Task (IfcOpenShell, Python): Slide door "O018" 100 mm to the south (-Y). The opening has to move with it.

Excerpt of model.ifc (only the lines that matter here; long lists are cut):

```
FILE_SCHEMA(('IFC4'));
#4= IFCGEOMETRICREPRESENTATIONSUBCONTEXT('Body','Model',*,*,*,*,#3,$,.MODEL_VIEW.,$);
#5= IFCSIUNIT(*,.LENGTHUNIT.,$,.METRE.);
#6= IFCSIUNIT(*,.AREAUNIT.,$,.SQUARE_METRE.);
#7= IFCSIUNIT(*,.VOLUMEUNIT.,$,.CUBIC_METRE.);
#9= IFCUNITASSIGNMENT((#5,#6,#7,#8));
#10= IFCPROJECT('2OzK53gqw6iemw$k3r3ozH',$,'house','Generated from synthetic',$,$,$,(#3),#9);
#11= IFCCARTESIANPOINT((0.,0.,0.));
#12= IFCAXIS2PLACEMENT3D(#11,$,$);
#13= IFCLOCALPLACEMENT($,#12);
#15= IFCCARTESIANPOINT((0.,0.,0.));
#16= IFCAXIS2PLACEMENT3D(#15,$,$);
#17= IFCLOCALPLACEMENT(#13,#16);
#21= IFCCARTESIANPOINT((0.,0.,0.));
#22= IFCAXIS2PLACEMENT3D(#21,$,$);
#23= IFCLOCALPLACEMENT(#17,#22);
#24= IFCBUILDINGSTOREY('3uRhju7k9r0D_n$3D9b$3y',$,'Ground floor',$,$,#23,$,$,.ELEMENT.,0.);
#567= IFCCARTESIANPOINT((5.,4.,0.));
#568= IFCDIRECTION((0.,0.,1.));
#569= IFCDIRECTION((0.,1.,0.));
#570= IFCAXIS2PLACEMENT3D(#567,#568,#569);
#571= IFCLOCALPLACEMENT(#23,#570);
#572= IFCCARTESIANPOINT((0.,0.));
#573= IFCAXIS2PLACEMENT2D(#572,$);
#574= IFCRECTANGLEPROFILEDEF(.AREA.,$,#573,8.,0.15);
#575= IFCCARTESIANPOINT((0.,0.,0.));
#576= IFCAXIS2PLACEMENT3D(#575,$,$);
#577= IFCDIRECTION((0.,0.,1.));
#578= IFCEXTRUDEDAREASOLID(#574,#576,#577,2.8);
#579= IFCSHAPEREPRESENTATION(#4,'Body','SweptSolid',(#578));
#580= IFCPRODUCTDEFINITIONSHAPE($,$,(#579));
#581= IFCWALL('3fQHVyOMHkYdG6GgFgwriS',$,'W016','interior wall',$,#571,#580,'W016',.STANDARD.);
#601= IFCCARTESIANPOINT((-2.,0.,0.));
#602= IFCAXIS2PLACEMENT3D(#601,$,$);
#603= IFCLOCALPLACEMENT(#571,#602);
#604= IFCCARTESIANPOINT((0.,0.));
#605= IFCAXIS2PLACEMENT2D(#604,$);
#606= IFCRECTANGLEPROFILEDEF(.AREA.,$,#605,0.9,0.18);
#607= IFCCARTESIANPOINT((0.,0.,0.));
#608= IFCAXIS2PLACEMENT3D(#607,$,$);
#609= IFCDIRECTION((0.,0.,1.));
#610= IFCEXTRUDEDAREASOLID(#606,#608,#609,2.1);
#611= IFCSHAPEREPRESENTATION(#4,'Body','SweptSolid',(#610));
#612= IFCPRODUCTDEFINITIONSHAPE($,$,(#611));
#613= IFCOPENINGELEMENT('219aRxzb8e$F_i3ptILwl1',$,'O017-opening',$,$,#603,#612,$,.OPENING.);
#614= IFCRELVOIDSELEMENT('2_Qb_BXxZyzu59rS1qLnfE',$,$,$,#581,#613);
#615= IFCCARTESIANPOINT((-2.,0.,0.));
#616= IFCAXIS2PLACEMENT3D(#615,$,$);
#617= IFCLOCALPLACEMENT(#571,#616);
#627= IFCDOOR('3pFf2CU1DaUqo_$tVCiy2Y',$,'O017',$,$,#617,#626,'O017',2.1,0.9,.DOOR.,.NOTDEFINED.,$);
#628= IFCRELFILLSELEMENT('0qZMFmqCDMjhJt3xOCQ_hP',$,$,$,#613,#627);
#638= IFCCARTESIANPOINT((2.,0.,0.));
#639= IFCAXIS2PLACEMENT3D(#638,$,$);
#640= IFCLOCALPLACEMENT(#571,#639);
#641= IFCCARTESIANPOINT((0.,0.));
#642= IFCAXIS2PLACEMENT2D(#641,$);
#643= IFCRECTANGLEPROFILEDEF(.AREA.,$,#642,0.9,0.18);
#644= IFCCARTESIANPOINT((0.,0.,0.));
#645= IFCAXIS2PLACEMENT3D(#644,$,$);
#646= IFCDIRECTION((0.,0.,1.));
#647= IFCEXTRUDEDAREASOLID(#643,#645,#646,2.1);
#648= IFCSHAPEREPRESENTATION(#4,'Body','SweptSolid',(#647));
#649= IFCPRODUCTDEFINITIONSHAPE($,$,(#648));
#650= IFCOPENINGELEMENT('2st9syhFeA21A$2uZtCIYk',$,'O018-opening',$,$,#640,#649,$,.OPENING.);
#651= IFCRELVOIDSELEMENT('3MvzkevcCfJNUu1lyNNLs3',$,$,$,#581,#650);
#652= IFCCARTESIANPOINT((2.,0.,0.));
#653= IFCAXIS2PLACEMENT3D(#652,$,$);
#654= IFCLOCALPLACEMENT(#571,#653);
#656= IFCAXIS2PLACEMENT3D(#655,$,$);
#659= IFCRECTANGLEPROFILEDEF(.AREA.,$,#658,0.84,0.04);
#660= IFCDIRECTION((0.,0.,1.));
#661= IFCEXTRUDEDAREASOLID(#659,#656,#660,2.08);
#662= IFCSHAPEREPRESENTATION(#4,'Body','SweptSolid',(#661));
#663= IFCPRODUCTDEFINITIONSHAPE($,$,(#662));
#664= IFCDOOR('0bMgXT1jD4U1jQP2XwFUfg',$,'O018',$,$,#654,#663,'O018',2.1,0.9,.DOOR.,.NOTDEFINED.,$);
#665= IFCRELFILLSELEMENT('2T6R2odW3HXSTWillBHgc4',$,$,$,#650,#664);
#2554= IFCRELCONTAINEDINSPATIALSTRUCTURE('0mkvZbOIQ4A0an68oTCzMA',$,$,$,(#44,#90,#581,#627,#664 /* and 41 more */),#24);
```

```python
import ifcopenshell
import ifcopenshell.api.geometry
import ifcopenshell.util.placement

model = ifcopenshell.open("model.ifc")

door = model.by_id(664)
opening = door.FillsVoids[0].RelatingOpeningElement
wall = opening.VoidsElements[0].RelatingBuildingElement

wall_matrix = ifcopenshell.util.placement.get_local_placement(wall.ObjectPlacement)
shift = wall_matrix[:3, 0] * -0.1
before = ifcopenshell.util.placement.get_local_placement(door.ObjectPlacement)[:3, 3].copy()

# The door is not placed relative to its opening, so move both.
for product in (opening, door):
    matrix = ifcopenshell.util.placement.get_local_placement(product.ObjectPlacement)
    matrix[:3, 3] += shift
    ifcopenshell.api.geometry.edit_object_placement(model, product=product, matrix=matrix, is_si=False)

after = ifcopenshell.util.placement.get_local_placement(door.ObjectPlacement)[:3, 3]
print("door moved by", (after - before).round(3) + 0.0)

model.write("model_v2.ifc")
```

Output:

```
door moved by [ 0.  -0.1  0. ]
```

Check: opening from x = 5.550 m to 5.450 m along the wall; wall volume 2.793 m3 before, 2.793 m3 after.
